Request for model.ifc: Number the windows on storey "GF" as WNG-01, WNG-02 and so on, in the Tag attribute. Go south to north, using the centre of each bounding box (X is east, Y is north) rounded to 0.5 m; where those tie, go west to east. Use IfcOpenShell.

First a look at what the model holds.

```python
import ifcopenshell
import ifcopenshell.util.element
import ifcopenshell.util.placement

model = ifcopenshell.open("model.ifc")
print(model.schema)
storey = next(s for s in model.by_type("IfcBuildingStorey") if s.Name == "GF")
windows = [e for e in ifcopenshell.util.element.get_decomposition(storey) if e.is_a("IfcWindow")]
for e in sorted(windows, key=lambda e: e.id()):
    origin = ifcopenshell.util.placement.get_local_placement(e.ObjectPlacement)[:3, 3]
    print(e.id(), e.Tag, e.Name, origin.round(2) + 0.0, sep=" | ")
```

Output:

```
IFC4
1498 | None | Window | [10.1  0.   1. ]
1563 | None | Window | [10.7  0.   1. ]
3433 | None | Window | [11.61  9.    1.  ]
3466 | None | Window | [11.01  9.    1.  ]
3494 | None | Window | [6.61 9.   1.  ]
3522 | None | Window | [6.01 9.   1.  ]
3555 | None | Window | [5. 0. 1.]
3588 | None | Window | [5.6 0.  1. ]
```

```python
import ifcopenshell
import ifcopenshell.geom
import ifcopenshell.util.element
import ifcopenshell.util.shape

model = ifcopenshell.open("model.ifc")
settings = ifcopenshell.geom.settings()
settings.set("use-world-coords", True)


def centre(element):
    shape = ifcopenshell.geom.create_shape(settings, element)
    return ifcopenshell.util.shape.get_bbox_centroid(shape.geometry)


storey = next(s for s in model.by_type("IfcBuildingStorey") if s.Name == "GF")
windows = [e for e in ifcopenshell.util.element.get_decomposition(storey) if e.is_a("IfcWindow")]

# Insertion points can sit at a corner or the storey origin, so sort by the geometry (in metres).
centres = {e: centre(e) for e in windows}
windows.sort(key=lambda e: (round(centres[e][1] / 0.5), centres[e][0]))

for i, e in enumerate(windows, start=1):
    number = f"WNG-{i:02d}"
    e.Tag = number
    print(e.id(), number)

model.write("model_v2.ifc")
```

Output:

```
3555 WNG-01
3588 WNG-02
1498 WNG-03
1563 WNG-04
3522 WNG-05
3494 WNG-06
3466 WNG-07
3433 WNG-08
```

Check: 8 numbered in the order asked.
